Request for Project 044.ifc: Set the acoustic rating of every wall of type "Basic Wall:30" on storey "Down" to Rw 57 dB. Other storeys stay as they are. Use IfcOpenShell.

First a look at what the model holds.

```python
import ifcopenshell
import ifcopenshell.util.element

model = ifcopenshell.open("Project 044.ifc")
print(model.schema)
storey = next(s for s in model.by_type("IfcBuildingStorey") if s.Name == "Down")
walls = [e for e in ifcopenshell.util.element.get_decomposition(storey) if e.is_a("IfcWall")]
seen = {}
for e in walls:
    element_type = ifcopenshell.util.element.get_type(e)
    key = (element_type.Name if element_type != e and element_type else None, ifcopenshell.util.element.get_pset(e, "Pset_WallCommon", "AcousticRating"))
    seen[key] = seen.get(key, 0) + 1
for (name, value), count in sorted(seen.items(), key=str):
    print(count, "x", name, "|", value)
```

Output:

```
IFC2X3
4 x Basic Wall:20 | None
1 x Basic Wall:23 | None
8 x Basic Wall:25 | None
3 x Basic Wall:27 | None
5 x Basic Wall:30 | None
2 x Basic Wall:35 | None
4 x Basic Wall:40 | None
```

```python
import ifcopenshell
import ifcopenshell.api.pset
import ifcopenshell.util.element

model = ifcopenshell.open("Project 044.ifc")

storey = next(s for s in model.by_type("IfcBuildingStorey") if s.Name == "Down")
walls = [e for e in ifcopenshell.util.element.get_decomposition(storey) if e.is_a("IfcWall")]

count = 0
for e in walls:
    element_type = ifcopenshell.util.element.get_type(e)
    if element_type in (None, e) or element_type.Name != "Basic Wall:30":
        continue
    # add_pset returns the element's existing set when there is one.
    pset = ifcopenshell.api.pset.add_pset(model, product=e, name="Pset_WallCommon")
    ifcopenshell.api.pset.edit_pset(model, pset=pset, properties={"AcousticRating": "Rw 57 dB"})
    count += 1

print(count, "walls updated")

model.write("Project 044_edited.ifc")
```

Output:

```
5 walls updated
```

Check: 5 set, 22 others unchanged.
